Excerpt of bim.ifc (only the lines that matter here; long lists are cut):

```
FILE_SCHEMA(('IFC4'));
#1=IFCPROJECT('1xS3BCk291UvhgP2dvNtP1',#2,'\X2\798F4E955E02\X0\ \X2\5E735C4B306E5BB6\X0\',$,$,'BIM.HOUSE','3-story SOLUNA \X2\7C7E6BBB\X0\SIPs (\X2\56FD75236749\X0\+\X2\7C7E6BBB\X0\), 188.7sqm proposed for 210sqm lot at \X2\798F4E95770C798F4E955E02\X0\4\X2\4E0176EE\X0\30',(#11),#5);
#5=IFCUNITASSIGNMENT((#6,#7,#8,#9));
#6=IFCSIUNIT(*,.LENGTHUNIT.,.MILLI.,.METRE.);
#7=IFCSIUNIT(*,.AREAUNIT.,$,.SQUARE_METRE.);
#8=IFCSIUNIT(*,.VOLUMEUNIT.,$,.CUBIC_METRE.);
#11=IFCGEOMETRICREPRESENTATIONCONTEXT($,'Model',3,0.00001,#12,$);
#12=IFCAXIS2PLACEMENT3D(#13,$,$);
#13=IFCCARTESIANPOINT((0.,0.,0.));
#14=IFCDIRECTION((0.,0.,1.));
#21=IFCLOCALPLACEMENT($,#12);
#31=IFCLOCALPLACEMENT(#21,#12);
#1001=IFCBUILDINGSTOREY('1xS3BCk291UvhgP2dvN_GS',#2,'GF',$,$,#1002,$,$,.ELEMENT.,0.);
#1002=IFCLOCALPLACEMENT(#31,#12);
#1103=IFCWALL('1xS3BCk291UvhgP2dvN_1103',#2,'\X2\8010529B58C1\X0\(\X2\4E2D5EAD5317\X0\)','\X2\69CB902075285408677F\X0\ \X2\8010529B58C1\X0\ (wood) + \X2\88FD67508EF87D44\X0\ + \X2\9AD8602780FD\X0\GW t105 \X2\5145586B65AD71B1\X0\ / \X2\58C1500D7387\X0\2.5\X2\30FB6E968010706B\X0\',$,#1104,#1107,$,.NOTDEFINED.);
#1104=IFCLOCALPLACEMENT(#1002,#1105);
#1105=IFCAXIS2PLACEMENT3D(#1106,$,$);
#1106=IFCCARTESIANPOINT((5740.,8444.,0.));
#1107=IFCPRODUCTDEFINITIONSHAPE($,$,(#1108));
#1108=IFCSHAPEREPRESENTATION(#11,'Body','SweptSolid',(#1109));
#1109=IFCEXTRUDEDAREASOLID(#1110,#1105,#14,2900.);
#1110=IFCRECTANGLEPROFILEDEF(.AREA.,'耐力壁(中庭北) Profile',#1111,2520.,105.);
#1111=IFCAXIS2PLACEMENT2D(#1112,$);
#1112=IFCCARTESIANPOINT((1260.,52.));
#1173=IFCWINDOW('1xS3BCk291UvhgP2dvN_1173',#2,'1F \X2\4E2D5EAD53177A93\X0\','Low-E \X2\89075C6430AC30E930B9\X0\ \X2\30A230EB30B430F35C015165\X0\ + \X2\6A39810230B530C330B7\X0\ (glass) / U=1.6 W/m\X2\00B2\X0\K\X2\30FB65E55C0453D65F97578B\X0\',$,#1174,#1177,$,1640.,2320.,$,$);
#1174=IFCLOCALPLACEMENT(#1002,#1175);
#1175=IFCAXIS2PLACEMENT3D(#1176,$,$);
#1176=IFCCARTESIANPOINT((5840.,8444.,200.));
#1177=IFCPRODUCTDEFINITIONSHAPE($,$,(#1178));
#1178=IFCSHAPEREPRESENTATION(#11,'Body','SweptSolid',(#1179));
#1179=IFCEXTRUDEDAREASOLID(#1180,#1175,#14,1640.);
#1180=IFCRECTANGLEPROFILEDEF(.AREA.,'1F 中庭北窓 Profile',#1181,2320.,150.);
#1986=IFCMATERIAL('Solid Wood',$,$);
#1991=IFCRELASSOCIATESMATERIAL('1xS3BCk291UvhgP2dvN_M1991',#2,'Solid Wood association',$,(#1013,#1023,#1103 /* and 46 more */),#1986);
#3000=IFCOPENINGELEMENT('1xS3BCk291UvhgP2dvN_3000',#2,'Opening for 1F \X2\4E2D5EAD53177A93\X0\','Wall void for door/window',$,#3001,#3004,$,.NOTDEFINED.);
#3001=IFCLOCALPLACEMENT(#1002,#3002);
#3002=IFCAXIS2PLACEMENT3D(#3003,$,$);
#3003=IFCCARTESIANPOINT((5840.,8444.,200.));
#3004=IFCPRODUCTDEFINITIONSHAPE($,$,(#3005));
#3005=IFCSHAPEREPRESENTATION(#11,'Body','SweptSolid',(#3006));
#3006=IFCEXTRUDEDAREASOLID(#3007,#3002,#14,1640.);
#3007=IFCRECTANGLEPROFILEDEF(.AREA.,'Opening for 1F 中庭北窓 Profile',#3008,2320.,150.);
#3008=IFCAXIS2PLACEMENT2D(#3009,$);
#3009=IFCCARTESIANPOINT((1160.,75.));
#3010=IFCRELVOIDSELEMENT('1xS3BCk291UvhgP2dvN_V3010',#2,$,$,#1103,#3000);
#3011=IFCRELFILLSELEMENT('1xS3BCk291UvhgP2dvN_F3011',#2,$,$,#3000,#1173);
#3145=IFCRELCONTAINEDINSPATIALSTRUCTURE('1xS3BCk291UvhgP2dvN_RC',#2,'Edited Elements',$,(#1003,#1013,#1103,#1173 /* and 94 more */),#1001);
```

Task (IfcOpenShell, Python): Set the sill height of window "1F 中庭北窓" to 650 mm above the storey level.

```python
import numpy as np
import ifcopenshell
import ifcopenshell.api.geometry
import ifcopenshell.geom
import ifcopenshell.util.element
import ifcopenshell.util.placement
import ifcopenshell.util.shape
import ifcopenshell.util.unit

model = ifcopenshell.open("bim.ifc")
unit_scale = ifcopenshell.util.unit.calculate_unit_scale(model)

window = model.by_guid("1xS3BCk291UvhgP2dvN_1173")
opening = window.FillsVoids[0].RelatingOpeningElement
storey = ifcopenshell.util.element.get_container(window, ifc_class="IfcBuildingStorey")
level = ifcopenshell.util.placement.get_local_placement(storey.ObjectPlacement)[2, 3]

# The opening's origin need not be at the sill, so measure its lowest point.
shape = ifcopenshell.geom.create_shape(ifcopenshell.geom.settings(), opening)
bottom = ifcopenshell.util.shape.get_shape_bottom_elevation(shape, shape.geometry) / unit_scale
dz = level + 0.65 / unit_scale - bottom

shift = np.array([0.0, 0.0, dz])
# The window is not placed relative to its opening, so move both.
for product in (opening, window):
    matrix = ifcopenshell.util.placement.get_local_placement(product.ObjectPlacement)
    matrix[:3, 3] += shift
    ifcopenshell.api.geometry.edit_object_placement(model, product=product, matrix=matrix, is_si=False)

print(f"moved by {dz * unit_scale:+.3f} m")

model.write("bim_edited.ifc")
```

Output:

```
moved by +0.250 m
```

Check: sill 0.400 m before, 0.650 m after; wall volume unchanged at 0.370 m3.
